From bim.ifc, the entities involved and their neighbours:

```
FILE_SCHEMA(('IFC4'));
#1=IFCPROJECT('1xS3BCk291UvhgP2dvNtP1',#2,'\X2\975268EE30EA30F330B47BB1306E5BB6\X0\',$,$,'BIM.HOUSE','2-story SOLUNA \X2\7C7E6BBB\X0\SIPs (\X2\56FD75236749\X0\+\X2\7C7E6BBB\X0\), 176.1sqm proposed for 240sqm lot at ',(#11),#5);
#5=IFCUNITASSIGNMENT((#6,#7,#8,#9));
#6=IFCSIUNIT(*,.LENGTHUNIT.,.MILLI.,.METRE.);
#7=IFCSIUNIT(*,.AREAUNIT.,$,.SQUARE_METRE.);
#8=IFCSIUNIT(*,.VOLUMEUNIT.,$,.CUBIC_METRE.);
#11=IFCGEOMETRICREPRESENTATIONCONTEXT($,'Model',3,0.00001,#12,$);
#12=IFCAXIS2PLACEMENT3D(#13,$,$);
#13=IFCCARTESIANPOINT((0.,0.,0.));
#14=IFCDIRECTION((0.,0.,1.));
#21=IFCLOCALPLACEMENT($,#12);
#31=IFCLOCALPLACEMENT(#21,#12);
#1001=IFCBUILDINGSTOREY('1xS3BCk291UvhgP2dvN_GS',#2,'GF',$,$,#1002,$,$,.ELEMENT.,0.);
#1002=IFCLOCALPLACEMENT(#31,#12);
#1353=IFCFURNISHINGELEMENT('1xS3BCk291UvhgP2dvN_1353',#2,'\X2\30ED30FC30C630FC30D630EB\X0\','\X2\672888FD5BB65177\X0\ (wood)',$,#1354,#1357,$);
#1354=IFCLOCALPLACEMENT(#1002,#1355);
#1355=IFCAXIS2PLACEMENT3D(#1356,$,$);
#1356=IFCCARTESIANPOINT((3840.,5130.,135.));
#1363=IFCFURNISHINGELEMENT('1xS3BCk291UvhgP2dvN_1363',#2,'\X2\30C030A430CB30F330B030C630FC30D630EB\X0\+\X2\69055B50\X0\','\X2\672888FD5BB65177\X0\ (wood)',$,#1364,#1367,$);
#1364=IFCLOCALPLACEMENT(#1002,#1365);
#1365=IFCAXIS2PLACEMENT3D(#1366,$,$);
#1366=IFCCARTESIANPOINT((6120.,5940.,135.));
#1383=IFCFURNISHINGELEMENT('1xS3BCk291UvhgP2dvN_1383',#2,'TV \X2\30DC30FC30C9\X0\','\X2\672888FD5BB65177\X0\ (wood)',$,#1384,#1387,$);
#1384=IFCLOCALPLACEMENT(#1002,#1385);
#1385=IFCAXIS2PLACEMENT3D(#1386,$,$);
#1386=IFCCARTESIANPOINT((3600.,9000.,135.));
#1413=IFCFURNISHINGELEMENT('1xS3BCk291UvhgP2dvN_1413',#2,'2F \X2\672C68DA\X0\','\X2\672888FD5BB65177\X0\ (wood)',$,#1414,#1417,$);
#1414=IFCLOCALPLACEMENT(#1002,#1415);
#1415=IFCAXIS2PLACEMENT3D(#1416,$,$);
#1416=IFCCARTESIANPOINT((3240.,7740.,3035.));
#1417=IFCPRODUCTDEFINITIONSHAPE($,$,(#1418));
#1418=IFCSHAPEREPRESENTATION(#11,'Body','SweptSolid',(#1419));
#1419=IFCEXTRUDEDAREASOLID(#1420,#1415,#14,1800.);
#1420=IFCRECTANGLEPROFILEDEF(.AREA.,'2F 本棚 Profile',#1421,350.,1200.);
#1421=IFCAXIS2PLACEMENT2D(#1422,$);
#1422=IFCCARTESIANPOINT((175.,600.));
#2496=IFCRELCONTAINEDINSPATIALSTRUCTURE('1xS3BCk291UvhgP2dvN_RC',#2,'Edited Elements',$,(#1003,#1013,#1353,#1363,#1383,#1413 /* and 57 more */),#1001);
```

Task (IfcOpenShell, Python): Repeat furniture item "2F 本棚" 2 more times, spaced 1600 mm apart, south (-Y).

```python
import numpy as np
import ifcopenshell
import ifcopenshell.api.geometry
import ifcopenshell.api.root
import ifcopenshell.util.element
import ifcopenshell.util.placement

model = ifcopenshell.open("bim.ifc")


def reuse_history(source, copy):
    """copy_class also copies each property set's owner history, people and application; keep the originals."""
    for rel in copy.IsDefinedBy:
        if rel.is_a("IfcRelDefinesByProperties") and (history := rel.RelatingPropertyDefinition.OwnerHistory):
            rel.RelatingPropertyDefinition.OwnerHistory = source.OwnerHistory
            ifcopenshell.util.element.remove_deep2(model, history)


source = model.by_id(1413)
base = ifcopenshell.util.placement.get_local_placement(source.ObjectPlacement)
step = np.array([0.0, -1.0, 0.0]) * 1600.0

for i in range(1, 3):
    copy = ifcopenshell.api.root.copy_class(model, product=source)
    copy.Representation = ifcopenshell.util.element.copy_deep(
        model, source.Representation, exclude=["IfcGeometricRepresentationContext", "IfcRepresentationMap"]
    )
    reuse_history(source, copy)
    matrix = base.copy()
    matrix[:3, 3] += i * step
    print("added at", matrix[:3, 3].round(3) + 0.0)
    ifcopenshell.api.geometry.edit_object_placement(model, product=copy, matrix=matrix, is_si=False)

model.write("bim_updated.ifc")
```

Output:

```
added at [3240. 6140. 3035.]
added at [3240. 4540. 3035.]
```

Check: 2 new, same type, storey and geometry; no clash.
